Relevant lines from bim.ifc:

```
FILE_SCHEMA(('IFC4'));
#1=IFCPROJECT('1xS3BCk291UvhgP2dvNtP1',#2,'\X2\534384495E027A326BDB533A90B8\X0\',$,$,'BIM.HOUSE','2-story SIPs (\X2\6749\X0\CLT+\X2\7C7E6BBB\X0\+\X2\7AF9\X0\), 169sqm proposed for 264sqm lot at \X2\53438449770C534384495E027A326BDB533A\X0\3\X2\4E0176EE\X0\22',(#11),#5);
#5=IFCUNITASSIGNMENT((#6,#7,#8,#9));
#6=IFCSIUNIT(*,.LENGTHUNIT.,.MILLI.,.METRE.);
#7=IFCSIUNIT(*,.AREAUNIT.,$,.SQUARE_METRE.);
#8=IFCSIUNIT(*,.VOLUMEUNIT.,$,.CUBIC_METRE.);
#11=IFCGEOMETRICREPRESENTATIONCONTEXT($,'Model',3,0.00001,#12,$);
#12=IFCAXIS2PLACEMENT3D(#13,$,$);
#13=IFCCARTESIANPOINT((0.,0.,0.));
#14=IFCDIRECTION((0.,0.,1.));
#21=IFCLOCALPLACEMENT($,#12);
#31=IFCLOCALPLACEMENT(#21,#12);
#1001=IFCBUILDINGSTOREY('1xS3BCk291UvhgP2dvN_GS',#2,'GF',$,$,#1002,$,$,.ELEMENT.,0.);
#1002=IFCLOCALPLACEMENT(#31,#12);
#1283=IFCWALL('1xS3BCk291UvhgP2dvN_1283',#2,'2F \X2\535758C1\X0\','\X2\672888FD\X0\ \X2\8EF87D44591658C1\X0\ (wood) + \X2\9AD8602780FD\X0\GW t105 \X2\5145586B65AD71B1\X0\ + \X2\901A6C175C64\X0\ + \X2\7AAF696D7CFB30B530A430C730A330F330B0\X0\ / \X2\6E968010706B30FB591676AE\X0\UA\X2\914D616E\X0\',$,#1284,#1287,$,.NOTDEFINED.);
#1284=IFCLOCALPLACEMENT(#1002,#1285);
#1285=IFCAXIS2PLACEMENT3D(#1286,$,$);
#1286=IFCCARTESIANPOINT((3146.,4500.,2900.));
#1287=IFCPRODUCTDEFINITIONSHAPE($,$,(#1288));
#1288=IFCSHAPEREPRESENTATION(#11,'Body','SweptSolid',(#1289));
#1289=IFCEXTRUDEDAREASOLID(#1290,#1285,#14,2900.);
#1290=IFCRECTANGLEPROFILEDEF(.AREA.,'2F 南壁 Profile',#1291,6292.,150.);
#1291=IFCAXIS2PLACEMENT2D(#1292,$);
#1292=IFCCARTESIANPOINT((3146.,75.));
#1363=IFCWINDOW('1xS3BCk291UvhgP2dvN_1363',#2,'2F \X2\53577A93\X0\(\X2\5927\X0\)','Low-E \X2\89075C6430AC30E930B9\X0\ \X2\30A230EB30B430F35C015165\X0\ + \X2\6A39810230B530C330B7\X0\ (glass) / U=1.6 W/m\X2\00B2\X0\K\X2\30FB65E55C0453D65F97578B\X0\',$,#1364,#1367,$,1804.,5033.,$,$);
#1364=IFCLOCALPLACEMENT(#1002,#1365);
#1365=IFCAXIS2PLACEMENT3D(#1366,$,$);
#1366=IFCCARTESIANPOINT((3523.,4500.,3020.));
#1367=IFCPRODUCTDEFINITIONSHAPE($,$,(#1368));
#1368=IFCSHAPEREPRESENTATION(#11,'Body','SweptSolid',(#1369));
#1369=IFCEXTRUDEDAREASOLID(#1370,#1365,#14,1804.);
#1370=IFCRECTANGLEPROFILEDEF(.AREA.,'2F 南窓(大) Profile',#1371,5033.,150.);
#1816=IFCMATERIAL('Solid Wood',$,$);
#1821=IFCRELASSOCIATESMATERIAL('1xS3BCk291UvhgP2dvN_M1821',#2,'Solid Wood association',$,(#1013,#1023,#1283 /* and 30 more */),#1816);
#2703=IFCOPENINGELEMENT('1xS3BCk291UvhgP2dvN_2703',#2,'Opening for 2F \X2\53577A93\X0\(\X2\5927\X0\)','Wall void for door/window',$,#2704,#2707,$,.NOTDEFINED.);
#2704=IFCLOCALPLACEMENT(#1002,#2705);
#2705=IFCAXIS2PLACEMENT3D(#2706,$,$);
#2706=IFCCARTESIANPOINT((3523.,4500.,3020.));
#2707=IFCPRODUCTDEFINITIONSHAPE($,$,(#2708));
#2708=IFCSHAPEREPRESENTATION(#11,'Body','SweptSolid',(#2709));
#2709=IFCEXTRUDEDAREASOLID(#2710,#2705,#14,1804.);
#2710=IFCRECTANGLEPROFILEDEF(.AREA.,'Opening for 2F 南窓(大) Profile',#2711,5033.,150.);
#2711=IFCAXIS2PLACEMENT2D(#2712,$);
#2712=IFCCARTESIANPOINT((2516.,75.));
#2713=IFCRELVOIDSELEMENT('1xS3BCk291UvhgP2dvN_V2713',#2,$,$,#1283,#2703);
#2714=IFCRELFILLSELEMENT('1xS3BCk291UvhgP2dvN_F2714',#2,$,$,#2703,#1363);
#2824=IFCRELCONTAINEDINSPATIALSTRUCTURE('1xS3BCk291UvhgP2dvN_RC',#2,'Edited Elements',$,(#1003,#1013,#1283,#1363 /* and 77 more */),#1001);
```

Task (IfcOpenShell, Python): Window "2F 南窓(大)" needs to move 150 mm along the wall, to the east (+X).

```python
import ifcopenshell
import ifcopenshell.api.geometry
import ifcopenshell.util.placement
import ifcopenshell.util.unit

model = ifcopenshell.open("bim.ifc")
unit_scale = ifcopenshell.util.unit.calculate_unit_scale(model)

window = model.by_guid("1xS3BCk291UvhgP2dvN_1363")
opening = window.FillsVoids[0].RelatingOpeningElement
wall = opening.VoidsElements[0].RelatingBuildingElement

wall_matrix = ifcopenshell.util.placement.get_local_placement(wall.ObjectPlacement)
shift = wall_matrix[:3, 0] * 0.15 / unit_scale
before = ifcopenshell.util.placement.get_local_placement(window.ObjectPlacement)[:3, 3].copy()

# The window is not placed relative to its opening, so move both.
for product in (opening, window):
    matrix = ifcopenshell.util.placement.get_local_placement(product.ObjectPlacement)
    matrix[:3, 3] += shift
    ifcopenshell.api.geometry.edit_object_placement(model, product=product, matrix=matrix, is_si=False)

after = ifcopenshell.util.placement.get_local_placement(window.ObjectPlacement)[:3, 3]
print("window moved by", (after - before).round(3) + 0.0)

model.write("bim_rev.ifc")
```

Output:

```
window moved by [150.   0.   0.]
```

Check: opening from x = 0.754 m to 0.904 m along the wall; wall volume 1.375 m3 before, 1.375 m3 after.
